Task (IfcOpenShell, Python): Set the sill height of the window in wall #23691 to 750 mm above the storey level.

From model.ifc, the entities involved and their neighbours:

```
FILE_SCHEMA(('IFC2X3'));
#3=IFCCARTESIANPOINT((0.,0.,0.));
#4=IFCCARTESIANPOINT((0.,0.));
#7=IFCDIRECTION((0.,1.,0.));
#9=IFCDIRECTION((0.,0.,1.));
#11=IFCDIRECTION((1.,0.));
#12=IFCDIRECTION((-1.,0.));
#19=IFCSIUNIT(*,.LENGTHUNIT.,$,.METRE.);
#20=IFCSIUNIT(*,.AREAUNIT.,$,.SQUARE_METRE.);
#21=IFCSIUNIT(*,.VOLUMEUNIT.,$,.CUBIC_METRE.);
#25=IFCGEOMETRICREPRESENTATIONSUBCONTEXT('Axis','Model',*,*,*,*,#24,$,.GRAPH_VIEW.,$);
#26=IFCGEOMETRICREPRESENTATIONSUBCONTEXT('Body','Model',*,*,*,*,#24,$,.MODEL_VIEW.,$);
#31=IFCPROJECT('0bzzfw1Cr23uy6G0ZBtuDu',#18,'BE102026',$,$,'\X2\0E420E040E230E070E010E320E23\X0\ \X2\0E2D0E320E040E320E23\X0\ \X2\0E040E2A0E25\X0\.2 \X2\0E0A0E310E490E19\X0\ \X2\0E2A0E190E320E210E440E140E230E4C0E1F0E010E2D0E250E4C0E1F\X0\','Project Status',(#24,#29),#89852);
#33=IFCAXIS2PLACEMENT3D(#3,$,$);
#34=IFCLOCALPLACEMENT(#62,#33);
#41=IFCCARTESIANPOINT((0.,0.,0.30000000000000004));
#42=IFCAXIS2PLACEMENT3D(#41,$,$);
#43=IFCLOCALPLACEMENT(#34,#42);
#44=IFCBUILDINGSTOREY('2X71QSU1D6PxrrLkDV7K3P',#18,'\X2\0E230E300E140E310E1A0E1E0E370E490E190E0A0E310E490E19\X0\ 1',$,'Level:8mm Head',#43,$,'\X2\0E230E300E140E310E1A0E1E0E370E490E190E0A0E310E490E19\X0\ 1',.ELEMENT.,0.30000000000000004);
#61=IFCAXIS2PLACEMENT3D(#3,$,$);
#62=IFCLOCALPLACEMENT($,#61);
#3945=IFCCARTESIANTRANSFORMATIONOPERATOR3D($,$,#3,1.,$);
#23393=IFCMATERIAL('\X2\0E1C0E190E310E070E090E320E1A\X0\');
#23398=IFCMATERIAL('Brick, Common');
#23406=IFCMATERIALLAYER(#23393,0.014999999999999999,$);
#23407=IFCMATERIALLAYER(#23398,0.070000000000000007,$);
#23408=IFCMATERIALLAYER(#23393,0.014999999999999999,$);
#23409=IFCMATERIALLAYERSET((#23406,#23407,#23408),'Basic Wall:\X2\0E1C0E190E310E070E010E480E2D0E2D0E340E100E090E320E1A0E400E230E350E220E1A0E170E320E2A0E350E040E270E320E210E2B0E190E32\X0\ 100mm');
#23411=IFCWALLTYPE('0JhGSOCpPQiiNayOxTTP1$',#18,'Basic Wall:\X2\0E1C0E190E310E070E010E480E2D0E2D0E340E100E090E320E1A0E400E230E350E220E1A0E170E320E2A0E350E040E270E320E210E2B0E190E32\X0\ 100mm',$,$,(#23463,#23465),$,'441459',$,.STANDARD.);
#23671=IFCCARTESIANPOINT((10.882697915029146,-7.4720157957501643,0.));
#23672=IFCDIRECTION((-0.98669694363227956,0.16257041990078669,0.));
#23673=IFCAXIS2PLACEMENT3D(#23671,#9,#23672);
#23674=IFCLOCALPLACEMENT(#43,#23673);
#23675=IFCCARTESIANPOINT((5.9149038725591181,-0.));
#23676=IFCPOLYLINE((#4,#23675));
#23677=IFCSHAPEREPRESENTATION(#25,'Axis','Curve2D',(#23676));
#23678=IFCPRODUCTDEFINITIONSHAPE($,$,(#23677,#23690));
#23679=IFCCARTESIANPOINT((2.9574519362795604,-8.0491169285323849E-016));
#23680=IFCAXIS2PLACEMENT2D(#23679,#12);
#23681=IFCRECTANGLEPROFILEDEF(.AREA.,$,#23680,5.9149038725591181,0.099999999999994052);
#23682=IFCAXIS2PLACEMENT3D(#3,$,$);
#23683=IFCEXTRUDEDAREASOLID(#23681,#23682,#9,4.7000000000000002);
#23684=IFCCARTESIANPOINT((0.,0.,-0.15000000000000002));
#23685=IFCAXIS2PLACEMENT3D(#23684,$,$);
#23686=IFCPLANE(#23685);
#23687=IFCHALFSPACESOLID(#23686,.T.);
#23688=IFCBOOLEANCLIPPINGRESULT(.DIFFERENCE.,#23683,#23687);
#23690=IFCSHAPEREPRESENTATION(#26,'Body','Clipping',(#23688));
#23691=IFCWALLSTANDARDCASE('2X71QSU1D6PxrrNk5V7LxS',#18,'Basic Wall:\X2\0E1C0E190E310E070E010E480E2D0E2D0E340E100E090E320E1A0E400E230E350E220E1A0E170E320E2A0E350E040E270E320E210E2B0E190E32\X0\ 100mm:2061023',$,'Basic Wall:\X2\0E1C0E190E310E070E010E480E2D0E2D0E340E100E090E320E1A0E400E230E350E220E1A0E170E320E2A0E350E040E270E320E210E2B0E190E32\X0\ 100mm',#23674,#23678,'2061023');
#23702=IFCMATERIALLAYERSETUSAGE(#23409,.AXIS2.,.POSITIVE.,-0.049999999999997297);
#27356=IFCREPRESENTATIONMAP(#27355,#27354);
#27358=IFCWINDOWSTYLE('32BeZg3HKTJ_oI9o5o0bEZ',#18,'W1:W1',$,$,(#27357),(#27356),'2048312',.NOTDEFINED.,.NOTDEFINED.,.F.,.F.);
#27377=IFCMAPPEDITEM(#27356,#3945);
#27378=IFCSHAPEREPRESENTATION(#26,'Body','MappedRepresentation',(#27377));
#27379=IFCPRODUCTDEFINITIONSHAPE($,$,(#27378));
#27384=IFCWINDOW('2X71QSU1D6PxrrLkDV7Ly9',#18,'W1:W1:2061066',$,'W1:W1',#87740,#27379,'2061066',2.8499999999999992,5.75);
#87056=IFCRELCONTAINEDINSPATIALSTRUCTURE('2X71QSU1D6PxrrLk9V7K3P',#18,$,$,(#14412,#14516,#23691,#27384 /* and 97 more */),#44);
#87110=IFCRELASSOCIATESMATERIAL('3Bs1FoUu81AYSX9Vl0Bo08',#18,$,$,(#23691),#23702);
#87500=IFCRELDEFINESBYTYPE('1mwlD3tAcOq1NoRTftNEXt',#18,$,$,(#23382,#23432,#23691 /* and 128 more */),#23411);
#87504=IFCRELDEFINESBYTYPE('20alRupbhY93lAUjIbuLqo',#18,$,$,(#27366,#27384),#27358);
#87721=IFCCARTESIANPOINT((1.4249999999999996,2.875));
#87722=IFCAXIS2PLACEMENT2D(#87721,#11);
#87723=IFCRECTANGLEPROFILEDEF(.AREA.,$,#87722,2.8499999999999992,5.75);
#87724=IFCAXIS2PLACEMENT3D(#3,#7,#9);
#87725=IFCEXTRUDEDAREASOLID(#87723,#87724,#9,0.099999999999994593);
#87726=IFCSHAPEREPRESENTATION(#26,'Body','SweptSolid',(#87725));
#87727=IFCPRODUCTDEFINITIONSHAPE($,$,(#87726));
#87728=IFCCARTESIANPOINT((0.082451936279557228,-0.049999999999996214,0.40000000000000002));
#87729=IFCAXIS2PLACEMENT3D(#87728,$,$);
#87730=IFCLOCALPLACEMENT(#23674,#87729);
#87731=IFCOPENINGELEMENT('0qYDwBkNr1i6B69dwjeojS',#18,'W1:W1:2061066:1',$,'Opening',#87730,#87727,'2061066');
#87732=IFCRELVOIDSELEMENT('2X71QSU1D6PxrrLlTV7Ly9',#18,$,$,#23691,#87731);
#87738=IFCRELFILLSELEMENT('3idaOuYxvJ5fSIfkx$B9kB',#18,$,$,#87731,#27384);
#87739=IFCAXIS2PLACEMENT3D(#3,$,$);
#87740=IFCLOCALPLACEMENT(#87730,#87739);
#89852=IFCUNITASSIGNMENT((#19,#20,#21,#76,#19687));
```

```python
import numpy as np
import ifcopenshell
import ifcopenshell.api.geometry
import ifcopenshell.geom
import ifcopenshell.util.element
import ifcopenshell.util.placement
import ifcopenshell.util.shape
import ifcopenshell.util.unit

model = ifcopenshell.open("model.ifc")
unit_scale = ifcopenshell.util.unit.calculate_unit_scale(model)

window = model.by_guid("2X71QSU1D6PxrrLkDV7Ly9")
opening = window.FillsVoids[0].RelatingOpeningElement
storey = ifcopenshell.util.element.get_container(window, ifc_class="IfcBuildingStorey")
level = ifcopenshell.util.placement.get_local_placement(storey.ObjectPlacement)[2, 3]

# The opening's origin need not be at the sill, so measure its lowest point.
shape = ifcopenshell.geom.create_shape(ifcopenshell.geom.settings(), opening)
bottom = ifcopenshell.util.shape.get_shape_bottom_elevation(shape, shape.geometry) / unit_scale
dz = level + 0.75 / unit_scale - bottom

shift = np.array([0.0, 0.0, dz])
# The window is placed relative to its opening, so it follows when the opening moves.
matrix = ifcopenshell.util.placement.get_local_placement(opening.ObjectPlacement)
matrix[:3, 3] += shift
ifcopenshell.api.geometry.edit_object_placement(
    model, product=opening, matrix=matrix, is_si=False, should_transform_children=True
)

print(f"moved by {dz * unit_scale:+.3f} m")

model.write("model_v2.ifc")
```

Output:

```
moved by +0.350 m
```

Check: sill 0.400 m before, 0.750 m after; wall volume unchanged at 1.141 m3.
